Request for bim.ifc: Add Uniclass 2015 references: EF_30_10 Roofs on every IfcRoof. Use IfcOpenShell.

First a look at what the model holds.

```python
import ifcopenshell

model = ifcopenshell.open("bim.ifc")
print(model.schema)
print("classifications:", [c.Name for c in model.by_type("IfcClassification")])
for ifc_class in ("IfcDoor", "IfcRoof", "IfcStair", "IfcWall", "IfcWindow"):
    print(ifc_class, len(model.by_type(ifc_class)))
```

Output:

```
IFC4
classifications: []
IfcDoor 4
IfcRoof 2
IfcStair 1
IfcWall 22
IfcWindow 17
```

```python
import ifcopenshell
import ifcopenshell.api.classification

model = ifcopenshell.open("bim.ifc")

system = ifcopenshell.api.classification.add_classification(model, classification="Uniclass 2015")

codes = {
    "IfcRoof": ("EF_30_10", "Roofs"),
}
for ifc_class, (code, name) in codes.items():
    products = model.by_type(ifc_class)
    ifcopenshell.api.classification.add_reference(
        model, products=products, classification=system, identification=code, name=name
    )
    print(code, len(products))

model.write("bim_v2.ifc")
```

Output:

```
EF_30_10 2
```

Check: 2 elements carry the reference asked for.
